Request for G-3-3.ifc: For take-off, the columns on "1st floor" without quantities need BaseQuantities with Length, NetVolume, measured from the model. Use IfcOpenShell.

First a look at what the model holds.

```python
import ifcopenshell
import ifcopenshell.util.element
import ifcopenshell.util.unit

model = ifcopenshell.open("G-3-3.ifc")
print(model.schema)
for unit_type in ("LENGTHUNIT", "AREAUNIT", "VOLUMEUNIT"):
    print(unit_type, ifcopenshell.util.unit.calculate_unit_scale(model, unit_type))
storey = next(s for s in model.by_type("IfcBuildingStorey") if s.Name == "1st floor")
columns = [e for e in ifcopenshell.util.element.get_decomposition(storey) if e.is_a("IfcColumn")]
for e in sorted(columns, key=lambda e: e.id()):
    print(e.id(), e.is_a(), e.Name, list(ifcopenshell.util.element.get_psets(e, qtos_only=True)), sep=" | ")
```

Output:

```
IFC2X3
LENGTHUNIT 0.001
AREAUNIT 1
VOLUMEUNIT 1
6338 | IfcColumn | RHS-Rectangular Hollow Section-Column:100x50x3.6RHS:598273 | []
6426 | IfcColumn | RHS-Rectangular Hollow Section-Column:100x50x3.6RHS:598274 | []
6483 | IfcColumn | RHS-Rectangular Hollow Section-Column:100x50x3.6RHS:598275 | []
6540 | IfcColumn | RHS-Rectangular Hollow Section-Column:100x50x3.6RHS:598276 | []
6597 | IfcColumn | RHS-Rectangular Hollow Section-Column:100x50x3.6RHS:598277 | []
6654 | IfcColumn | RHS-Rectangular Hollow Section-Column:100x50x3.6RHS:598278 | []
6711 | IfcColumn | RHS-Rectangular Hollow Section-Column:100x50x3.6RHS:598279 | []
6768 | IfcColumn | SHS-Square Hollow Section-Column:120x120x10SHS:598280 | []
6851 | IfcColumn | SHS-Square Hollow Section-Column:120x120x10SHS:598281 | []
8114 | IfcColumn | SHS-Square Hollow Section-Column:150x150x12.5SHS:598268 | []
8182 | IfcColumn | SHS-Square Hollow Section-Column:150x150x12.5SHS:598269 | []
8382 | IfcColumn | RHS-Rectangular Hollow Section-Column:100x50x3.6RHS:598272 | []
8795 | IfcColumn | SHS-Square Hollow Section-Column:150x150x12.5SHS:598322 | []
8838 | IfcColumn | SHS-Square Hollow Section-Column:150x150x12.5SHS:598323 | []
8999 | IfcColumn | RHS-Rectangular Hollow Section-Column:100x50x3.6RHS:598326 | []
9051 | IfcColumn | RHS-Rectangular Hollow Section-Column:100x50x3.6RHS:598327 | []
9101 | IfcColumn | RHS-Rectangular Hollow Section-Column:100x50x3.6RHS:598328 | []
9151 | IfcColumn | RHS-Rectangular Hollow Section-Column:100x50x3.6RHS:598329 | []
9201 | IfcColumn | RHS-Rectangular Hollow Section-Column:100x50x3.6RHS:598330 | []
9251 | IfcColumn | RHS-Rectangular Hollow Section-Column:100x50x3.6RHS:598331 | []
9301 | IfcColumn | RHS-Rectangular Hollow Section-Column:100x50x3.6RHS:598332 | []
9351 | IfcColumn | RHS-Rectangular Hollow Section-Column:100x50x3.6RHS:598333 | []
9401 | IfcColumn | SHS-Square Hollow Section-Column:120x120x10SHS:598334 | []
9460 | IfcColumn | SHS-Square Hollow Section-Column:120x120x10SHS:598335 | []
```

```python
import ifcopenshell
import ifcopenshell.api.pset
import ifcopenshell.geom
import ifcopenshell.util.element
import ifcopenshell.util.shape
import ifcopenshell.util.unit

model = ifcopenshell.open("G-3-3.ifc")
unit_scale = ifcopenshell.util.unit.calculate_unit_scale(model)
volume_scale = ifcopenshell.util.unit.calculate_unit_scale(model, "VOLUMEUNIT")
settings = ifcopenshell.geom.settings()

storey = next(s for s in model.by_type("IfcBuildingStorey") if s.Name == "1st floor")
columns = [e for e in ifcopenshell.util.element.get_decomposition(storey) if e.is_a("IfcColumn")]

for e in sorted(columns, key=lambda e: e.id()):
    if ifcopenshell.util.element.get_psets(e, qtos_only=True, should_inherit=False):
        continue
    # Geometry comes back in metres, in the element's own axes.
    shape = ifcopenshell.geom.create_shape(settings, e)
    values = {
        "Length": ifcopenshell.util.shape.get_z(shape.geometry) / unit_scale,
        "NetVolume": ifcopenshell.util.shape.get_volume(shape.geometry) / volume_scale,
    }
    qto = ifcopenshell.api.pset.add_qto(model, product=e, name="BaseQuantities")
    ifcopenshell.api.pset.edit_qto(model, qto=qto, properties=values)
    print(e.id(), {k: round(v, 3) for k, v in values.items()})

model.write("G-3-3_v2.ifc")
```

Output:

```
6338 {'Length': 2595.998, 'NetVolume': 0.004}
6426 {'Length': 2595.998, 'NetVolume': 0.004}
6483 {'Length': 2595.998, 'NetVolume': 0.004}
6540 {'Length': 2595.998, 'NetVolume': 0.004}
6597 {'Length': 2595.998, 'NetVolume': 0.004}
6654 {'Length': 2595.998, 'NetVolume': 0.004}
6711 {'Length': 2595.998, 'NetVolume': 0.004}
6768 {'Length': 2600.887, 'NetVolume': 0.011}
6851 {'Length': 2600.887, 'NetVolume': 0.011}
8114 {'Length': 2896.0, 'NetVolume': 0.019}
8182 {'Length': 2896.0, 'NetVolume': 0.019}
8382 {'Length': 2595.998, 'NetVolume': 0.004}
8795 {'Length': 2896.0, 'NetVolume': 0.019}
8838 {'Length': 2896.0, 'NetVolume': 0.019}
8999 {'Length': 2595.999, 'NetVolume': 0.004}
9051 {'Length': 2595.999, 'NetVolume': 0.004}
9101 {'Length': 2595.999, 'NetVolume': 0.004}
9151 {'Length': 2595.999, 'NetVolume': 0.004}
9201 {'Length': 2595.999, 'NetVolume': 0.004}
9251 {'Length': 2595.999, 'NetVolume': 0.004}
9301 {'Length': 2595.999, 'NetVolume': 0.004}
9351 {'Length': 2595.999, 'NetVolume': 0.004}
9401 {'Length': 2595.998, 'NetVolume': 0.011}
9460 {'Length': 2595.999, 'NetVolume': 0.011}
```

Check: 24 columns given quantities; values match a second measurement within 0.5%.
